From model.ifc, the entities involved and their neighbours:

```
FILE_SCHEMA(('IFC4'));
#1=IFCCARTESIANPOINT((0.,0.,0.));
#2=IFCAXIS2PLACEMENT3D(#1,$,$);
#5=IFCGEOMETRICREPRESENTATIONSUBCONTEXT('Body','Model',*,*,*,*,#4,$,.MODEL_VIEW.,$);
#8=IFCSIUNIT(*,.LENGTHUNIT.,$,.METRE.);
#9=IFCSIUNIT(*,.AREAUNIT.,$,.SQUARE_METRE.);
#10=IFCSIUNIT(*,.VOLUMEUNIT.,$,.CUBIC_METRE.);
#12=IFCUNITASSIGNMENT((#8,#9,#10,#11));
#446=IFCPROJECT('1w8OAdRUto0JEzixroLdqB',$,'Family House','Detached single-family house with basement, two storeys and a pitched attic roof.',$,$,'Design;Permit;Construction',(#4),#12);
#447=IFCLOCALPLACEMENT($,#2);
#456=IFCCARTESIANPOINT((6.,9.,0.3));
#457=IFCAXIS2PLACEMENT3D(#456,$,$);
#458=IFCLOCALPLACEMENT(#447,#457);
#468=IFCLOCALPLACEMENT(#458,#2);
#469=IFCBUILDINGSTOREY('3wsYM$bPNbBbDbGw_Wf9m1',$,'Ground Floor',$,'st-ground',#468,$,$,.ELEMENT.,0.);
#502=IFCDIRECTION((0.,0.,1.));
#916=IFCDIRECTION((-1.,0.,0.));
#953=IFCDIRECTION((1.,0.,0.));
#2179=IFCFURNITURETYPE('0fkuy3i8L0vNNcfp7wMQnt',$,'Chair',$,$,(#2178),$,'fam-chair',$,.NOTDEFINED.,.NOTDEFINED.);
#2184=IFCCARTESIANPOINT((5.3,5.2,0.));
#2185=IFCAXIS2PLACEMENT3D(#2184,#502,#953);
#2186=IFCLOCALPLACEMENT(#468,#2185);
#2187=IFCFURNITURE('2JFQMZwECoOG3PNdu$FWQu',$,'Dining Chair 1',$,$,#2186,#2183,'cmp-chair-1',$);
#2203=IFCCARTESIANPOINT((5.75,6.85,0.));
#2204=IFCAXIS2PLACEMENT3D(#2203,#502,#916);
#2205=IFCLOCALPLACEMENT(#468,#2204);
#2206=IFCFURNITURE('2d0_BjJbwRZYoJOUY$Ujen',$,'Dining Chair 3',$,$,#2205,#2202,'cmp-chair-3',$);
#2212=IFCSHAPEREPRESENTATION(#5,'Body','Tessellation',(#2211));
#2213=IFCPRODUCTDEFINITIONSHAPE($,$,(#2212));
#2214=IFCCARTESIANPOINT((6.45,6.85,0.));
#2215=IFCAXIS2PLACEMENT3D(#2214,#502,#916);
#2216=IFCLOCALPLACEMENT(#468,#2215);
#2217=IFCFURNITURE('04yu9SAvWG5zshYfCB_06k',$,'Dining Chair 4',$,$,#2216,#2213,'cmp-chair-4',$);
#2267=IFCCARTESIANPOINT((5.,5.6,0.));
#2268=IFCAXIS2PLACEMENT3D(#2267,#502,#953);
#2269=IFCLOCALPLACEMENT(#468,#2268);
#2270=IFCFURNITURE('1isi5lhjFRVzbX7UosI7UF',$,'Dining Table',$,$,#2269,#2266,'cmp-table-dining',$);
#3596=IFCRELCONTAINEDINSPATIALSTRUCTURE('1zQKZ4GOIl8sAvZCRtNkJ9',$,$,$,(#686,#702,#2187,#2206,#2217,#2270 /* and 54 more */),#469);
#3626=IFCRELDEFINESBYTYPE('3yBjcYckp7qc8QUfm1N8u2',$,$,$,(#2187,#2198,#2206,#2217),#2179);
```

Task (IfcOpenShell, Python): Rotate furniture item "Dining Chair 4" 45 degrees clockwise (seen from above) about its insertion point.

```python
import ifcopenshell
import ifcopenshell.api.geometry
import ifcopenshell.util.placement

model = ifcopenshell.open("model.ifc")

item = model.by_id(2217)
matrix = ifcopenshell.util.placement.get_local_placement(item.ObjectPlacement)
matrix = matrix @ ifcopenshell.util.placement.rotation(-45, "Z")
ifcopenshell.api.geometry.edit_object_placement(model, product=item, matrix=matrix, is_si=False)

print(ifcopenshell.util.placement.get_local_placement(item.ObjectPlacement).round(3) + 0.0)

model.write("model_updated.ifc")
```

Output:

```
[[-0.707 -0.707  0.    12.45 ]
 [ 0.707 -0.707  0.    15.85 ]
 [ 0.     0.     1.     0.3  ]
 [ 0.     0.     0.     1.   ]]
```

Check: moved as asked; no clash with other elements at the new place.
